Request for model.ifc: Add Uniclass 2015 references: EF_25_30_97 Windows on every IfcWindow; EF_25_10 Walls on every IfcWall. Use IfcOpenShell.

First a look at what the model holds.

```python
import ifcopenshell

model = ifcopenshell.open("model.ifc")
print(model.schema)
print("classifications:", [c.Name for c in model.by_type("IfcClassification")])
for ifc_class in ("IfcDoor", "IfcRoof", "IfcStair", "IfcWall", "IfcWindow"):
    print(ifc_class, len(model.by_type(ifc_class)))
```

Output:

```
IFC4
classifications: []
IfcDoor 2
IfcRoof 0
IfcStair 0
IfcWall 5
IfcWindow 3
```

```python
import ifcopenshell
import ifcopenshell.api.classification

model = ifcopenshell.open("model.ifc")

system = ifcopenshell.api.classification.add_classification(model, classification="Uniclass 2015")

codes = {
    "IfcWindow": ("EF_25_30_97", "Windows"),
    "IfcWall": ("EF_25_10", "Walls"),
}
for ifc_class, (code, name) in codes.items():
    products = model.by_type(ifc_class)
    ifcopenshell.api.classification.add_reference(
        model, products=products, classification=system, identification=code, name=name
    )
    print(code, len(products))

model.write("model_v2.ifc")
```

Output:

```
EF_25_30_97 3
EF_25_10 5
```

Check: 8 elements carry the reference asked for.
